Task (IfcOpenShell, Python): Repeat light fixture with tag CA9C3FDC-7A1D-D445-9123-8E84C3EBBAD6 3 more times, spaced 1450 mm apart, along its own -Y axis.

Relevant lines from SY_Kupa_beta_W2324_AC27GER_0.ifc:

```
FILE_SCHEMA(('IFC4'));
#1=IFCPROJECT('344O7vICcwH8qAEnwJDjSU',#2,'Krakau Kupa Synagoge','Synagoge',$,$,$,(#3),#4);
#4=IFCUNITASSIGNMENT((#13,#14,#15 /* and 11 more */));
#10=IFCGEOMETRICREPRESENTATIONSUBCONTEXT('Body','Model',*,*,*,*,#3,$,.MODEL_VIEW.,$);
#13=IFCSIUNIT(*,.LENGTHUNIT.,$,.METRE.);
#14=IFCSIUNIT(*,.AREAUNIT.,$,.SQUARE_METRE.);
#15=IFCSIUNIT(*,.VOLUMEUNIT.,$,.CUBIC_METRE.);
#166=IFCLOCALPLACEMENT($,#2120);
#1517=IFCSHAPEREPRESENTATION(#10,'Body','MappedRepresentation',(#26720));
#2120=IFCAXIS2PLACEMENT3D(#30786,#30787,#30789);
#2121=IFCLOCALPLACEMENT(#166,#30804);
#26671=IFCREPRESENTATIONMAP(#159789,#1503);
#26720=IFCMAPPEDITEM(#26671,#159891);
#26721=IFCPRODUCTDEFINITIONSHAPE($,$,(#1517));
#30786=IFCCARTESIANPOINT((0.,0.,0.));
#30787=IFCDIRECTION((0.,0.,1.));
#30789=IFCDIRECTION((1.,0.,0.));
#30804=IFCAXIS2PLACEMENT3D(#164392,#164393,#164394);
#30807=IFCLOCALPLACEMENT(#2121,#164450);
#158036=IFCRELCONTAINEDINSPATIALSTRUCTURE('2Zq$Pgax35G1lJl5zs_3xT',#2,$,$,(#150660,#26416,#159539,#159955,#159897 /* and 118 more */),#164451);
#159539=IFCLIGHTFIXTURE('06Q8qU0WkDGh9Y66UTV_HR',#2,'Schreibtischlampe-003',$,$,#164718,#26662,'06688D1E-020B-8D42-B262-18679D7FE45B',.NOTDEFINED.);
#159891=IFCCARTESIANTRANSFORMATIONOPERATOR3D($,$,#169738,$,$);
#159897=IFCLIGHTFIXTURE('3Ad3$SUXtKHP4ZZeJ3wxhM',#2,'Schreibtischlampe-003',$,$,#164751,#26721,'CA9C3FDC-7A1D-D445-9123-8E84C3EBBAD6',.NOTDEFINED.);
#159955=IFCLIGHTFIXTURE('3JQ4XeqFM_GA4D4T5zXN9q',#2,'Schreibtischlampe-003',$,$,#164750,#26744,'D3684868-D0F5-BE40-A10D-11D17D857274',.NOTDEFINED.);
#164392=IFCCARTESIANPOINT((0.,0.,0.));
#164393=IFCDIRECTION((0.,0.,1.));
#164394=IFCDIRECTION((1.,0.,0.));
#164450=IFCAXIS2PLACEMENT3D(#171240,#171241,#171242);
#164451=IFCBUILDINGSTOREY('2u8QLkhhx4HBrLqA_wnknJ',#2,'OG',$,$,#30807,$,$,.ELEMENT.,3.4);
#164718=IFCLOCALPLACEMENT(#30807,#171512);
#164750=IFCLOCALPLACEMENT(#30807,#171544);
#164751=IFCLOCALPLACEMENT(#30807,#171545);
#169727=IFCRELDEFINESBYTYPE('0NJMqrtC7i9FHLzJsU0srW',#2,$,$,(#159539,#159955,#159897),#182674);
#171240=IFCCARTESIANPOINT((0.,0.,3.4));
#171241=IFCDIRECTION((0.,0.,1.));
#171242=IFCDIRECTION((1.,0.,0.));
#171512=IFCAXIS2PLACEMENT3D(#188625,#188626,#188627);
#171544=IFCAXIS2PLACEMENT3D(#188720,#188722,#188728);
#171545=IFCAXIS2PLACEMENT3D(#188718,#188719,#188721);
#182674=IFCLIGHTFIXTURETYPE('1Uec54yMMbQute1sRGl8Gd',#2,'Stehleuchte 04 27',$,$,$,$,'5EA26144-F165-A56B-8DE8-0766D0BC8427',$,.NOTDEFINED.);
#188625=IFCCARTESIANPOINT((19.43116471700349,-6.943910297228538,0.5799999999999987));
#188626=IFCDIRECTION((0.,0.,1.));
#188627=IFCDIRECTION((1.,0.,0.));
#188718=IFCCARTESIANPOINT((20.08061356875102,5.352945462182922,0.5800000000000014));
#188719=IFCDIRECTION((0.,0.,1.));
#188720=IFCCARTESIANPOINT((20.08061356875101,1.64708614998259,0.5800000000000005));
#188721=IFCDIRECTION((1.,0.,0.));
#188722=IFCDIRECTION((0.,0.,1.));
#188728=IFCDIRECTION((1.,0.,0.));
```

```python
import ifcopenshell
import ifcopenshell.api.geometry
import ifcopenshell.api.root
import ifcopenshell.util.element
import ifcopenshell.util.placement

model = ifcopenshell.open("SY_Kupa_beta_W2324_AC27GER_0.ifc")


def reuse_history(source, copy):
    """copy_class also copies each property set's owner history, people and application; keep the originals."""
    for rel in copy.IsDefinedBy:
        if rel.is_a("IfcRelDefinesByProperties") and (history := rel.RelatingPropertyDefinition.OwnerHistory):
            rel.RelatingPropertyDefinition.OwnerHistory = source.OwnerHistory
            ifcopenshell.util.element.remove_deep2(model, history)


source = model.by_guid("3Ad3$SUXtKHP4ZZeJ3wxhM")
base = ifcopenshell.util.placement.get_local_placement(source.ObjectPlacement)
step = -base[:3, 1] * 1.45

for i in range(1, 4):
    copy = ifcopenshell.api.root.copy_class(model, product=source)
    copy.Representation = ifcopenshell.util.element.copy_deep(
        model, source.Representation, exclude=["IfcGeometricRepresentationContext", "IfcRepresentationMap"]
    )
    copy.Tag = None
    reuse_history(source, copy)
    matrix = base.copy()
    matrix[:3, 3] += i * step
    print("added at", matrix[:3, 3].round(3) + 0.0)
    ifcopenshell.api.geometry.edit_object_placement(model, product=copy, matrix=matrix, is_si=False)

model.write("SY_Kupa_beta_W2324_AC27GER_0_edited.ifc")
```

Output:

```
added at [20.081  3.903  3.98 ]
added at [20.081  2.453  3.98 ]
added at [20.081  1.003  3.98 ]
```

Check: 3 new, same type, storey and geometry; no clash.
